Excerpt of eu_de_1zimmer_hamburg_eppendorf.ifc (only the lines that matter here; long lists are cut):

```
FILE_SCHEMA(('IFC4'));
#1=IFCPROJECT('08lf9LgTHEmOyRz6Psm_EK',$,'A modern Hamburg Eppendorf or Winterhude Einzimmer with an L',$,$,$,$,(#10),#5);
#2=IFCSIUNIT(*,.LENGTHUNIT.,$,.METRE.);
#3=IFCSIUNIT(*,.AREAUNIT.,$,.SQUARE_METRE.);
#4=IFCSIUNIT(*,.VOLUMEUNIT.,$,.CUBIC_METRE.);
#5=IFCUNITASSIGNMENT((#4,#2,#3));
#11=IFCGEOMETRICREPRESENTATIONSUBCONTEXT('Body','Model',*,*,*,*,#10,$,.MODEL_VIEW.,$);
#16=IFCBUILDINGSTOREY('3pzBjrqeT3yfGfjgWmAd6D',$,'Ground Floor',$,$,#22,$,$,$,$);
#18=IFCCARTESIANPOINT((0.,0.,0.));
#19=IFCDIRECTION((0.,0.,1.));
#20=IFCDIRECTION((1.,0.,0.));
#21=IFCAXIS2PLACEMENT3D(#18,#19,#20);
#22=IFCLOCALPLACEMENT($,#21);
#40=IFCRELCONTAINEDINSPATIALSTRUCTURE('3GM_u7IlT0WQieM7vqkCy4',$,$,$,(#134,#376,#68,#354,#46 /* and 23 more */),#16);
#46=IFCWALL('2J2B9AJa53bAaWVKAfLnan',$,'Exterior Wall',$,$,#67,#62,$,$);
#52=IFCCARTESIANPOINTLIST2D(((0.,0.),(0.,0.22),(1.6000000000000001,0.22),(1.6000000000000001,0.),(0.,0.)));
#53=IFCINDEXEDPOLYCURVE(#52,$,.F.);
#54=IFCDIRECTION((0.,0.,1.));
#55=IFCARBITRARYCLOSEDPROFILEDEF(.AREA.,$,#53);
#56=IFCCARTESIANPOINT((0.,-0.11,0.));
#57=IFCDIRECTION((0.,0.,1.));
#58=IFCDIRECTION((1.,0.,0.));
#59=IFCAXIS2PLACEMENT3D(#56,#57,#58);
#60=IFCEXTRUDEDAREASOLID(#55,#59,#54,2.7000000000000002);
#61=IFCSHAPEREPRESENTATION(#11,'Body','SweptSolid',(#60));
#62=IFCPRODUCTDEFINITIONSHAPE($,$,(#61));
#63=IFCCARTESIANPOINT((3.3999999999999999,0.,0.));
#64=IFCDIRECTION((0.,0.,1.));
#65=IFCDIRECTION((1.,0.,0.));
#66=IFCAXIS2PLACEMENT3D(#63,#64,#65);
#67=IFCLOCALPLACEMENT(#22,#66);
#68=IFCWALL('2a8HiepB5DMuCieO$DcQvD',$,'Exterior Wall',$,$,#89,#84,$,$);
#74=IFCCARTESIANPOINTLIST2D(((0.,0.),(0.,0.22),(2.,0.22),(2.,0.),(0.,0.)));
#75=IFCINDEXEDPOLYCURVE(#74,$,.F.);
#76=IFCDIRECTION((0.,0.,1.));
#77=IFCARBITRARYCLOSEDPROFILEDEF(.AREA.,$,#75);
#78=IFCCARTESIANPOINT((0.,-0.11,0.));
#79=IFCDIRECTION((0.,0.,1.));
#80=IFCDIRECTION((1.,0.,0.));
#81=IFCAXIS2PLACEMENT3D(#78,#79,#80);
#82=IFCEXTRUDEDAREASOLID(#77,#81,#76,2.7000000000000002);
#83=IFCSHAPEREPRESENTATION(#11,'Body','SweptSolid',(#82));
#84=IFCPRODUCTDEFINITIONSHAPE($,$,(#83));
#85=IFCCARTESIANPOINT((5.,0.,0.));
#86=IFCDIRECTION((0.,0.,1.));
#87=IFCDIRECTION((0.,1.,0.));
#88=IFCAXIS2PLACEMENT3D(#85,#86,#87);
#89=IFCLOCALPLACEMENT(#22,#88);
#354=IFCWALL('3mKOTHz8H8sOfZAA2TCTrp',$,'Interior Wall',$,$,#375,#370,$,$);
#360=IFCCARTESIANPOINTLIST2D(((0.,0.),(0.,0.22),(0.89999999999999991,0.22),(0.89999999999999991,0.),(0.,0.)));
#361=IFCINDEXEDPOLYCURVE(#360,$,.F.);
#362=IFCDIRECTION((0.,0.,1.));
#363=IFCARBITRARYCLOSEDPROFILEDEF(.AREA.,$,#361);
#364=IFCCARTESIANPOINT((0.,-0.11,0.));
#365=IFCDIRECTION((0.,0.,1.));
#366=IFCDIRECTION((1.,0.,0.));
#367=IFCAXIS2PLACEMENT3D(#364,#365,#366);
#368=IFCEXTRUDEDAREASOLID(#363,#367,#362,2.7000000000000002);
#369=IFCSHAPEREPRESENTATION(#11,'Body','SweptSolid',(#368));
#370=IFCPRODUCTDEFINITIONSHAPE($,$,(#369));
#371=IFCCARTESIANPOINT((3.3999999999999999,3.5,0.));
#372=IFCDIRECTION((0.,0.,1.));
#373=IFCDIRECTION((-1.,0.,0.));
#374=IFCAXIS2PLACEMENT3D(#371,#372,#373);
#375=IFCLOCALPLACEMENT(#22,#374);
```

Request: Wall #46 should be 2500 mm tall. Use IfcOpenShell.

```python
import ifcopenshell
import ifcopenshell.geom
import ifcopenshell.util.representation
import ifcopenshell.util.shape
import ifcopenshell.util.unit

model = ifcopenshell.open("eu_de_1zimmer_hamburg_eppendorf.ifc")
unit_scale = ifcopenshell.util.unit.calculate_unit_scale(model)
settings = ifcopenshell.geom.settings()


def volume(element):
    """Net volume in cubic metres, openings subtracted."""
    shape = ifcopenshell.geom.create_shape(settings, element)
    return ifcopenshell.util.shape.get_volume(shape.geometry)


wall = model.by_guid("2J2B9AJa53bAaWVKAfLnan")
before = volume(wall)

body = ifcopenshell.util.representation.get_representation(wall, "Model", "Body")
solid = body.Items[0]
old_height = solid.Depth
solid.Depth = 2.5 / unit_scale
after = volume(wall)

print(f"height {old_height:g} -> {solid.Depth:g}, volume {before:.3f} -> {after:.3f} m3")

model.write("eu_de_1zimmer_hamburg_eppendorf-out.ifc")
```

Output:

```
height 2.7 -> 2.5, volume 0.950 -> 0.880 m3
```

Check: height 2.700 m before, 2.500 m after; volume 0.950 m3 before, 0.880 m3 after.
